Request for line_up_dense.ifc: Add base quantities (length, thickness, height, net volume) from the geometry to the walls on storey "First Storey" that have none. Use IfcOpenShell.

First a look at what the model holds.

```python
import ifcopenshell
import ifcopenshell.util.element
import ifcopenshell.util.unit

model = ifcopenshell.open("line_up_dense.ifc")
print(model.schema)
for unit_type in ("LENGTHUNIT", "AREAUNIT", "VOLUMEUNIT"):
    print(unit_type, ifcopenshell.util.unit.calculate_unit_scale(model, unit_type))
storey = next(s for s in model.by_type("IfcBuildingStorey") if s.Name == "First Storey")
walls = [e for e in ifcopenshell.util.element.get_decomposition(storey) if e.is_a("IfcWall")]
for e in sorted(walls, key=lambda e: e.id()):
    print(e.id(), e.is_a(), e.Name, list(ifcopenshell.util.element.get_psets(e, qtos_only=True)), sep=" | ")
```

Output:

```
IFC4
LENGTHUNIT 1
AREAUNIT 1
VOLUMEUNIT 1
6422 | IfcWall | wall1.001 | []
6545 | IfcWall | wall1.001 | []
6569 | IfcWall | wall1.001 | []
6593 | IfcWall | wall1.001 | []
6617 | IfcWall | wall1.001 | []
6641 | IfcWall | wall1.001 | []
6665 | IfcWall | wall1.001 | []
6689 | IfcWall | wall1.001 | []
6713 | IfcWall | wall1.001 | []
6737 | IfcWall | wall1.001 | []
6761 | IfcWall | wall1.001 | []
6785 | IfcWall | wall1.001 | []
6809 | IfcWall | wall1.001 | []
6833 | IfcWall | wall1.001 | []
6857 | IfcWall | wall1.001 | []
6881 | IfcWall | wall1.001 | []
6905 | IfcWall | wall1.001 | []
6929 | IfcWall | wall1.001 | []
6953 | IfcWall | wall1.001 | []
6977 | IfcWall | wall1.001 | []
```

```python
import ifcopenshell
import ifcopenshell.api.pset
import ifcopenshell.geom
import ifcopenshell.util.element
import ifcopenshell.util.shape
import ifcopenshell.util.unit

model = ifcopenshell.open("line_up_dense.ifc")
unit_scale = ifcopenshell.util.unit.calculate_unit_scale(model)
volume_scale = ifcopenshell.util.unit.calculate_unit_scale(model, "VOLUMEUNIT")
settings = ifcopenshell.geom.settings()

storey = next(s for s in model.by_type("IfcBuildingStorey") if s.Name == "First Storey")
walls = [e for e in ifcopenshell.util.element.get_decomposition(storey) if e.is_a("IfcWall")]

for e in sorted(walls, key=lambda e: e.id()):
    if ifcopenshell.util.element.get_psets(e, qtos_only=True, should_inherit=False):
        continue
    # Geometry comes back in metres, in the element's own axes.
    shape = ifcopenshell.geom.create_shape(settings, e)
    values = {
        "Length": ifcopenshell.util.shape.get_x(shape.geometry) / unit_scale,
        "Width": ifcopenshell.util.shape.get_y(shape.geometry) / unit_scale,
        "Height": ifcopenshell.util.shape.get_z(shape.geometry) / unit_scale,
        "NetVolume": ifcopenshell.util.shape.get_volume(shape.geometry) / volume_scale,
    }
    qto = ifcopenshell.api.pset.add_qto(model, product=e, name="Qto_WallBaseQuantities")
    ifcopenshell.api.pset.edit_qto(model, qto=qto, properties=values)
    print(e.id(), {k: round(v, 3) for k, v in values.items()})

model.write("line_up_dense_edited.ifc")
```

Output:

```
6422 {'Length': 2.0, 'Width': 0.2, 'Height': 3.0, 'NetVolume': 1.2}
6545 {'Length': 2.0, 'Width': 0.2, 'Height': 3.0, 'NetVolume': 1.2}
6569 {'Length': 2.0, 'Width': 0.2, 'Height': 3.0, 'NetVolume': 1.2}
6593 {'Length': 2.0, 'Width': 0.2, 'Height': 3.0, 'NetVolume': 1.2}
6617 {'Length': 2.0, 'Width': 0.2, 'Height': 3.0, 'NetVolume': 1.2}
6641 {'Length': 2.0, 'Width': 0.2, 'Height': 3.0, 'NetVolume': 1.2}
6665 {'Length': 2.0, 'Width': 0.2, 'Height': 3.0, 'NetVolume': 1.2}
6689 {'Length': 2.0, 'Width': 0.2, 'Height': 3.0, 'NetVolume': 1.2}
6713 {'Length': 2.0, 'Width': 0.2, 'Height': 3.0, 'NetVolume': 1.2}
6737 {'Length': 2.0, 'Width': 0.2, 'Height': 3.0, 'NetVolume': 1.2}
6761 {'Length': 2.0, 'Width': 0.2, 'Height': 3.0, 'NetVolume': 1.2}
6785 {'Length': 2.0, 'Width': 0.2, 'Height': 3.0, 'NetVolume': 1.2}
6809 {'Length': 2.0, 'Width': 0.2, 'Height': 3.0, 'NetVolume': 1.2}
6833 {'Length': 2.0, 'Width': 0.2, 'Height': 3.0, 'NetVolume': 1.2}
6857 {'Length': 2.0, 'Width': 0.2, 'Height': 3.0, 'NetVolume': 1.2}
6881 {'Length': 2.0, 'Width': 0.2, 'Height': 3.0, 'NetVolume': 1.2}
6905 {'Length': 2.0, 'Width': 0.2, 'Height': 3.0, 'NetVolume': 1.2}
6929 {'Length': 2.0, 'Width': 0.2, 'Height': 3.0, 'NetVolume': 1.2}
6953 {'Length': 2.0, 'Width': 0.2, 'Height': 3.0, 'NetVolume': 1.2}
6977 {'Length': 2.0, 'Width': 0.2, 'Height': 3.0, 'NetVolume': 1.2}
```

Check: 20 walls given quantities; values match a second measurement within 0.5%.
